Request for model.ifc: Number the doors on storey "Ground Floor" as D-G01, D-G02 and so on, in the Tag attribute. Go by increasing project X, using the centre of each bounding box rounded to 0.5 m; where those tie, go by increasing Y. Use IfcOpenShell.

First a look at what the model holds.

```python
import ifcopenshell
import ifcopenshell.util.element
import ifcopenshell.util.placement

model = ifcopenshell.open("model.ifc")
print(model.schema)
storey = next(s for s in model.by_type("IfcBuildingStorey") if s.Name == "Ground Floor")
doors = [e for e in ifcopenshell.util.element.get_decomposition(storey) if e.is_a("IfcDoor")]
for e in sorted(doors, key=lambda e: e.id()):
    origin = ifcopenshell.util.placement.get_local_placement(e.ObjectPlacement)[:3, 3]
    print(e.id(), e.Tag, e.Name, origin.round(2) + 0.0, sep=" | ")
```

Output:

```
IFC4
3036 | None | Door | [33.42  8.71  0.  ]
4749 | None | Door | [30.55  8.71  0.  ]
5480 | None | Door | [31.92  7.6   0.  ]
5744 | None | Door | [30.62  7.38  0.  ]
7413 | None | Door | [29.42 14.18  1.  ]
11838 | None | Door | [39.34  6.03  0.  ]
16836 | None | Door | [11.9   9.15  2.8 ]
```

```python
import ifcopenshell
import ifcopenshell.geom
import ifcopenshell.util.element
import ifcopenshell.util.shape

model = ifcopenshell.open("model.ifc")
settings = ifcopenshell.geom.settings()
settings.set("use-world-coords", True)


def centre(element):
    shape = ifcopenshell.geom.create_shape(settings, element)
    return ifcopenshell.util.shape.get_bbox_centroid(shape.geometry)


storey = next(s for s in model.by_type("IfcBuildingStorey") if s.Name == "Ground Floor")
doors = [e for e in ifcopenshell.util.element.get_decomposition(storey) if e.is_a("IfcDoor")]

# Insertion points can sit at a corner or the storey origin, so sort by the geometry (in metres).
centres = {e: centre(e) for e in doors}
doors.sort(key=lambda e: (round(centres[e][0] / 0.5), centres[e][1]))

for i, e in enumerate(doors, start=1):
    number = f"D-G{i:02d}"
    e.Tag = number
    print(e.id(), number)

model.write("model_edited.ifc")
```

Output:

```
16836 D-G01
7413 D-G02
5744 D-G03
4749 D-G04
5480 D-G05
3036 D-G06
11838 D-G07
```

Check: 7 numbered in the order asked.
